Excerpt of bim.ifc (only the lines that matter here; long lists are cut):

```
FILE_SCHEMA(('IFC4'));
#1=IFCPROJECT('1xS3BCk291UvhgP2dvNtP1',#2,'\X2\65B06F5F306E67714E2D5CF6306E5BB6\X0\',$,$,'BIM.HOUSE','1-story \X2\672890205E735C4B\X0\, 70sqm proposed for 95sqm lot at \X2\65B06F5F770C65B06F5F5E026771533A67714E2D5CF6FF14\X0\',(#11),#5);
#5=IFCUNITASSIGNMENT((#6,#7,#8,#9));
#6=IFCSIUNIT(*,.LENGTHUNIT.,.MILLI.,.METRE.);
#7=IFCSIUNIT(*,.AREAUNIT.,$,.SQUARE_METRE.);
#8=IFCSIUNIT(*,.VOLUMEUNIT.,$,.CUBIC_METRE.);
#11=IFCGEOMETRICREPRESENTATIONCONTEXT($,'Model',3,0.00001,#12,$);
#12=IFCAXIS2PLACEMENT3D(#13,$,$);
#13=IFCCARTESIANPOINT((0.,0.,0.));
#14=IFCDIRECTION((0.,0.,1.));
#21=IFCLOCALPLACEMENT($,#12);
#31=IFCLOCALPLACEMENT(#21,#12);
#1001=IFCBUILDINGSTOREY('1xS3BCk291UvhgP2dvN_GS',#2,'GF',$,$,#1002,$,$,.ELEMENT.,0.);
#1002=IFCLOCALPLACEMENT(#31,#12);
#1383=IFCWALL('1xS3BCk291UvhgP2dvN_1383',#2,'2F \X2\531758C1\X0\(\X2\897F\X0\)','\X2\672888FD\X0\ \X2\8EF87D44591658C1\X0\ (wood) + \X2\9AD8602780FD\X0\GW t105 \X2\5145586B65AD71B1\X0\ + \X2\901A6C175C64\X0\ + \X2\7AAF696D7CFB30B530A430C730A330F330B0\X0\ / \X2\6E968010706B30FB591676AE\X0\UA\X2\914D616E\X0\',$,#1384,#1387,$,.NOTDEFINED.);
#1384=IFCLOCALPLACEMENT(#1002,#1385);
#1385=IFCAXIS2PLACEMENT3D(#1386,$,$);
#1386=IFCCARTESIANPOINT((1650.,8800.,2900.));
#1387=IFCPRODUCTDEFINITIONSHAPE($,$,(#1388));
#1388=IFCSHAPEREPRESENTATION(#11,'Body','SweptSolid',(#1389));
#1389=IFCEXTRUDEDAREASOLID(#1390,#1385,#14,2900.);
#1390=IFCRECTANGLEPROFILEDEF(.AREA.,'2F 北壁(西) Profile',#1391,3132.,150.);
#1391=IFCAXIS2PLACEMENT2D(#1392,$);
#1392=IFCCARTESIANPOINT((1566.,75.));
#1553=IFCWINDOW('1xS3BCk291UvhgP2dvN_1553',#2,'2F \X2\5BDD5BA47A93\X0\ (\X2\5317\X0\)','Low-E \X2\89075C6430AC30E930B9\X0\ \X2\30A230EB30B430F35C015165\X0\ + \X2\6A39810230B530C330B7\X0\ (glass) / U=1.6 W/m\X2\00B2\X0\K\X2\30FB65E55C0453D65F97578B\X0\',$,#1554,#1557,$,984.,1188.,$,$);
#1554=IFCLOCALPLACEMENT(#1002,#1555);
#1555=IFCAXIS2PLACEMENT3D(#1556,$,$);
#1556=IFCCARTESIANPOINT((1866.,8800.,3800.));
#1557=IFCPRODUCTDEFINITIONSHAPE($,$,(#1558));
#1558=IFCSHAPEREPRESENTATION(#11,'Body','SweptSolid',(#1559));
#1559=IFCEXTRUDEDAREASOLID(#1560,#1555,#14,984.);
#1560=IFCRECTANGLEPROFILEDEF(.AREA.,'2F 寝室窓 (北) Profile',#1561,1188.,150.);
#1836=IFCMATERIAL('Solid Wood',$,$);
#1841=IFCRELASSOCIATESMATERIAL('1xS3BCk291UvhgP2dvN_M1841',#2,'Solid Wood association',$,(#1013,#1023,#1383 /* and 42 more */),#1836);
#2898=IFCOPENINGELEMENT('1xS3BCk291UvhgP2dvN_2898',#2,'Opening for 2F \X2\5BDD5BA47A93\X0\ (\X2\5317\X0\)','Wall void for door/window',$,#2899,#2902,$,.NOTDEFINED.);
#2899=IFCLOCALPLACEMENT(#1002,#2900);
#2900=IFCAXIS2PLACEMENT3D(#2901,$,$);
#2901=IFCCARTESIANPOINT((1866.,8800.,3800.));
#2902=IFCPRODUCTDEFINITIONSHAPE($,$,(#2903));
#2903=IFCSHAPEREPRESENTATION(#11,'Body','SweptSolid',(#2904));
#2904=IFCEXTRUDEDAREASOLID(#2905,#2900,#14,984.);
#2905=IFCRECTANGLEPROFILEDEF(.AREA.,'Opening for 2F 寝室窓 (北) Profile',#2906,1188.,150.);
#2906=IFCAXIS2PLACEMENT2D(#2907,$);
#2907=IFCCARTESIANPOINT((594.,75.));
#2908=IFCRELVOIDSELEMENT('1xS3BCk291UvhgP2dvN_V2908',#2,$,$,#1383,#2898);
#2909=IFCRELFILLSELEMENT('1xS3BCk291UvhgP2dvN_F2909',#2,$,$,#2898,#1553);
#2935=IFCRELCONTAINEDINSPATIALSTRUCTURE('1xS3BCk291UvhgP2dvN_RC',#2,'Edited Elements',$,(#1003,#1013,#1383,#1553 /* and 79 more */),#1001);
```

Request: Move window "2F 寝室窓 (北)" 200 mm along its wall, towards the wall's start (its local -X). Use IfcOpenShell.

```python
import ifcopenshell
import ifcopenshell.api.geometry
import ifcopenshell.util.placement
import ifcopenshell.util.unit

model = ifcopenshell.open("bim.ifc")
unit_scale = ifcopenshell.util.unit.calculate_unit_scale(model)

window = model.by_guid("1xS3BCk291UvhgP2dvN_1553")
opening = window.FillsVoids[0].RelatingOpeningElement
wall = opening.VoidsElements[0].RelatingBuildingElement

wall_matrix = ifcopenshell.util.placement.get_local_placement(wall.ObjectPlacement)
shift = wall_matrix[:3, 0] * -0.2 / unit_scale
before = ifcopenshell.util.placement.get_local_placement(window.ObjectPlacement)[:3, 3].copy()

# The window is not placed relative to its opening, so move both.
for product in (opening, window):
    matrix = ifcopenshell.util.placement.get_local_placement(product.ObjectPlacement)
    matrix[:3, 3] += shift
    ifcopenshell.api.geometry.edit_object_placement(model, product=product, matrix=matrix, is_si=False)

after = ifcopenshell.util.placement.get_local_placement(window.ObjectPlacement)[:3, 3]
print("window moved by", (after - before).round(3) + 0.0)

model.write("bim_edited.ifc")
```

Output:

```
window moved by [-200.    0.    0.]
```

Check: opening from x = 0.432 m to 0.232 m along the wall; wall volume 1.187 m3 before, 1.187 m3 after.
